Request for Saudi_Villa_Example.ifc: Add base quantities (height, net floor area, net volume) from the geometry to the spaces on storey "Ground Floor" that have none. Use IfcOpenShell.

First a look at what the model holds.

```python
import ifcopenshell
import ifcopenshell.util.element
import ifcopenshell.util.unit

model = ifcopenshell.open("Saudi_Villa_Example.ifc")
print(model.schema)
for unit_type in ("LENGTHUNIT", "AREAUNIT", "VOLUMEUNIT"):
    print(unit_type, ifcopenshell.util.unit.calculate_unit_scale(model, unit_type))
storey = next(s for s in model.by_type("IfcBuildingStorey") if s.Name == "Ground Floor")
spaces = [e for e in ifcopenshell.util.element.get_decomposition(storey) if e.is_a("IfcSpace")]
for e in sorted(spaces, key=lambda e: e.id()):
    print(e.id(), e.is_a(), e.Name, list(ifcopenshell.util.element.get_psets(e, qtos_only=True)), sep=" | ")
```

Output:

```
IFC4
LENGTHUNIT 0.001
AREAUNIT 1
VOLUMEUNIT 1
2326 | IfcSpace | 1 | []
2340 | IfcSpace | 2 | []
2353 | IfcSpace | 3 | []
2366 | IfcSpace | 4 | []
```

```python
import ifcopenshell
import ifcopenshell.api.pset
import ifcopenshell.geom
import ifcopenshell.util.element
import ifcopenshell.util.shape
import ifcopenshell.util.unit

model = ifcopenshell.open("Saudi_Villa_Example.ifc")
unit_scale = ifcopenshell.util.unit.calculate_unit_scale(model)
area_scale = ifcopenshell.util.unit.calculate_unit_scale(model, "AREAUNIT")
volume_scale = ifcopenshell.util.unit.calculate_unit_scale(model, "VOLUMEUNIT")
settings = ifcopenshell.geom.settings()

storey = next(s for s in model.by_type("IfcBuildingStorey") if s.Name == "Ground Floor")
spaces = [e for e in ifcopenshell.util.element.get_decomposition(storey) if e.is_a("IfcSpace")]

for e in sorted(spaces, key=lambda e: e.id()):
    if ifcopenshell.util.element.get_psets(e, qtos_only=True, should_inherit=False):
        continue
    # Geometry comes back in metres, in the element's own axes.
    shape = ifcopenshell.geom.create_shape(settings, e)
    values = {
        "Height": ifcopenshell.util.shape.get_z(shape.geometry) / unit_scale,
        "NetFloorArea": ifcopenshell.util.shape.get_footprint_area(shape.geometry) / area_scale,
        "NetVolume": ifcopenshell.util.shape.get_volume(shape.geometry) / volume_scale,
    }
    qto = ifcopenshell.api.pset.add_qto(model, product=e, name="Qto_SpaceBaseQuantities")
    ifcopenshell.api.pset.edit_qto(model, qto=qto, properties=values)
    print(e.id(), {k: round(v, 3) for k, v in values.items()})

model.write("Saudi_Villa_Example_edited.ifc")
```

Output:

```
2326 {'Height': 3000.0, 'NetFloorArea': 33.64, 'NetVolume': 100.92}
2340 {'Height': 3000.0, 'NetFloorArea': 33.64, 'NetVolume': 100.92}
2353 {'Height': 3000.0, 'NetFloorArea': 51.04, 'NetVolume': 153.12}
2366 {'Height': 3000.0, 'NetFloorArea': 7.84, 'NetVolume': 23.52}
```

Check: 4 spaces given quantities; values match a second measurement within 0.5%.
